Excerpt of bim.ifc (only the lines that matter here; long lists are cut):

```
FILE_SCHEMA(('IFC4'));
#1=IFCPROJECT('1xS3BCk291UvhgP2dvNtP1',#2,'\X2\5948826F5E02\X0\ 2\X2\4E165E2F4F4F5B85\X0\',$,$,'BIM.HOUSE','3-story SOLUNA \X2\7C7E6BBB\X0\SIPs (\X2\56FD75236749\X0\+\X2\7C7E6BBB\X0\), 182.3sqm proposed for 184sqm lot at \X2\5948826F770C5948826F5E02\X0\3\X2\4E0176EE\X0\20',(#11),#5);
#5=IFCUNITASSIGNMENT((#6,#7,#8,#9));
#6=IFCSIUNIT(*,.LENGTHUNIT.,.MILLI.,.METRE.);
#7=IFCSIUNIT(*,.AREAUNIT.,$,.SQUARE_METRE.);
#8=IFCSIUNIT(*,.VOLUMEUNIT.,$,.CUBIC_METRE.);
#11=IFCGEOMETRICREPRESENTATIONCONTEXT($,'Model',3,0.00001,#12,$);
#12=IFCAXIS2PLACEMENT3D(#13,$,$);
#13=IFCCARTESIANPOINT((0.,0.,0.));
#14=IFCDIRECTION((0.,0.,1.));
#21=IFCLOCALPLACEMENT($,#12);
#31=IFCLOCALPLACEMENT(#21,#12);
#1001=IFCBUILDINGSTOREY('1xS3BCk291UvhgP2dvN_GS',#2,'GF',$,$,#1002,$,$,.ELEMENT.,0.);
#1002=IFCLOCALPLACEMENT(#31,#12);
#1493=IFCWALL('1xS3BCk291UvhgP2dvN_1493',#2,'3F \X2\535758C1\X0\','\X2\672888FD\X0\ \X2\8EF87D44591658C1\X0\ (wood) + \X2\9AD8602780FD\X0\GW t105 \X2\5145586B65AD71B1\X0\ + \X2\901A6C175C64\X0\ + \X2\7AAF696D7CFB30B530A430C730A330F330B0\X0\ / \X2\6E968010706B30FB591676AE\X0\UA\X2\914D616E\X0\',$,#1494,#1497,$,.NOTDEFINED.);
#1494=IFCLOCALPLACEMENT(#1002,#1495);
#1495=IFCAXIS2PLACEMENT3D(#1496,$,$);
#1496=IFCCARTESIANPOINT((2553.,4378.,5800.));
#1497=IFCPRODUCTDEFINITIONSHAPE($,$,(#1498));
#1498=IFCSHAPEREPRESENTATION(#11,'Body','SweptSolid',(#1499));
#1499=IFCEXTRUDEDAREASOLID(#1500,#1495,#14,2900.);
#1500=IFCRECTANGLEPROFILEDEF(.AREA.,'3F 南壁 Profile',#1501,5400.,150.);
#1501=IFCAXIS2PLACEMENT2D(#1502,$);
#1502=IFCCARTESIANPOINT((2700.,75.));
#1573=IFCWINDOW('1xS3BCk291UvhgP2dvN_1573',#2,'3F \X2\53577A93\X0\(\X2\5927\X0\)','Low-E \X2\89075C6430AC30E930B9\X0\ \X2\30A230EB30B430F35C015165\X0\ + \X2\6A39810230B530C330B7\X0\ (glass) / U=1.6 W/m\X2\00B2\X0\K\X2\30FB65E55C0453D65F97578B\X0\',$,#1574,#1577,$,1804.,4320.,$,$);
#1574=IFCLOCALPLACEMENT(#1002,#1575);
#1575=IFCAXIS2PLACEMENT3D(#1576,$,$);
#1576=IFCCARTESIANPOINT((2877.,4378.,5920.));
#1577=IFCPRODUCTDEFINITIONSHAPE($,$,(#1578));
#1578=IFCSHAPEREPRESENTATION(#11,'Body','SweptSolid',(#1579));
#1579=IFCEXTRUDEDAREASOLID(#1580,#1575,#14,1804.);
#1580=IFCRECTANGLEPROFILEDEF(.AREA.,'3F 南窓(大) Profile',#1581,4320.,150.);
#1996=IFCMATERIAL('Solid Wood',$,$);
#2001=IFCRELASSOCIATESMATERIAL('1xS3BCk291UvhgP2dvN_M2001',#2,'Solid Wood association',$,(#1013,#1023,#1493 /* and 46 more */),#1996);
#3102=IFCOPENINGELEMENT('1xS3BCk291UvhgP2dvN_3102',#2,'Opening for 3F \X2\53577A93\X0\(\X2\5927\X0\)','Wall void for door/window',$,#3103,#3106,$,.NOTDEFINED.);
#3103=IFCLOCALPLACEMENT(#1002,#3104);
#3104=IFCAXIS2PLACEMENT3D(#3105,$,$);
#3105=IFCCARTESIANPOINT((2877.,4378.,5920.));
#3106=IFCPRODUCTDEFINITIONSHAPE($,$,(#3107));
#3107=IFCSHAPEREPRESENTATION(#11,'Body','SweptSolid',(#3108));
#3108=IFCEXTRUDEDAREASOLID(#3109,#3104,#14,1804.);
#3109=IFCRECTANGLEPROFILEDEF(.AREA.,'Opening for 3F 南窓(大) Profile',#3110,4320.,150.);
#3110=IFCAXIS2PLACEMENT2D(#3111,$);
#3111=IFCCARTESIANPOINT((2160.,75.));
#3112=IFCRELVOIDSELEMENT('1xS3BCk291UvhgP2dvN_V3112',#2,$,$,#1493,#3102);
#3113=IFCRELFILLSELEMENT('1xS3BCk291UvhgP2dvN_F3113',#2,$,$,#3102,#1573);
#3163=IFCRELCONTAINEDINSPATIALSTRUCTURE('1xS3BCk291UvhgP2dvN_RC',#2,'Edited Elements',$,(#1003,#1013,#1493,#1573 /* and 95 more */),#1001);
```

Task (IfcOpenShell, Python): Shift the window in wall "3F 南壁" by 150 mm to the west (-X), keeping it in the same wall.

```python
import ifcopenshell
import ifcopenshell.api.geometry
import ifcopenshell.util.placement

model = ifcopenshell.open("bim.ifc")

window = model.by_guid("1xS3BCk291UvhgP2dvN_1573")
opening = window.FillsVoids[0].RelatingOpeningElement
wall = opening.VoidsElements[0].RelatingBuildingElement

wall_matrix = ifcopenshell.util.placement.get_local_placement(wall.ObjectPlacement)
shift = wall_matrix[:3, 0] * -150.0
before = ifcopenshell.util.placement.get_local_placement(window.ObjectPlacement)[:3, 3].copy()

# The window is not placed relative to its opening, so move both.
for product in (opening, window):
    matrix = ifcopenshell.util.placement.get_local_placement(product.ObjectPlacement)
    matrix[:3, 3] += shift
    ifcopenshell.api.geometry.edit_object_placement(model, product=product, matrix=matrix, is_si=False)

after = ifcopenshell.util.placement.get_local_placement(window.ObjectPlacement)[:3, 3]
print("window moved by", (after - before).round(3) + 0.0)

model.write("bim-out.ifc")
```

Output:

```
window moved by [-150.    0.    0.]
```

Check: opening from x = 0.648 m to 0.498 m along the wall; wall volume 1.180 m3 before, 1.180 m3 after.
